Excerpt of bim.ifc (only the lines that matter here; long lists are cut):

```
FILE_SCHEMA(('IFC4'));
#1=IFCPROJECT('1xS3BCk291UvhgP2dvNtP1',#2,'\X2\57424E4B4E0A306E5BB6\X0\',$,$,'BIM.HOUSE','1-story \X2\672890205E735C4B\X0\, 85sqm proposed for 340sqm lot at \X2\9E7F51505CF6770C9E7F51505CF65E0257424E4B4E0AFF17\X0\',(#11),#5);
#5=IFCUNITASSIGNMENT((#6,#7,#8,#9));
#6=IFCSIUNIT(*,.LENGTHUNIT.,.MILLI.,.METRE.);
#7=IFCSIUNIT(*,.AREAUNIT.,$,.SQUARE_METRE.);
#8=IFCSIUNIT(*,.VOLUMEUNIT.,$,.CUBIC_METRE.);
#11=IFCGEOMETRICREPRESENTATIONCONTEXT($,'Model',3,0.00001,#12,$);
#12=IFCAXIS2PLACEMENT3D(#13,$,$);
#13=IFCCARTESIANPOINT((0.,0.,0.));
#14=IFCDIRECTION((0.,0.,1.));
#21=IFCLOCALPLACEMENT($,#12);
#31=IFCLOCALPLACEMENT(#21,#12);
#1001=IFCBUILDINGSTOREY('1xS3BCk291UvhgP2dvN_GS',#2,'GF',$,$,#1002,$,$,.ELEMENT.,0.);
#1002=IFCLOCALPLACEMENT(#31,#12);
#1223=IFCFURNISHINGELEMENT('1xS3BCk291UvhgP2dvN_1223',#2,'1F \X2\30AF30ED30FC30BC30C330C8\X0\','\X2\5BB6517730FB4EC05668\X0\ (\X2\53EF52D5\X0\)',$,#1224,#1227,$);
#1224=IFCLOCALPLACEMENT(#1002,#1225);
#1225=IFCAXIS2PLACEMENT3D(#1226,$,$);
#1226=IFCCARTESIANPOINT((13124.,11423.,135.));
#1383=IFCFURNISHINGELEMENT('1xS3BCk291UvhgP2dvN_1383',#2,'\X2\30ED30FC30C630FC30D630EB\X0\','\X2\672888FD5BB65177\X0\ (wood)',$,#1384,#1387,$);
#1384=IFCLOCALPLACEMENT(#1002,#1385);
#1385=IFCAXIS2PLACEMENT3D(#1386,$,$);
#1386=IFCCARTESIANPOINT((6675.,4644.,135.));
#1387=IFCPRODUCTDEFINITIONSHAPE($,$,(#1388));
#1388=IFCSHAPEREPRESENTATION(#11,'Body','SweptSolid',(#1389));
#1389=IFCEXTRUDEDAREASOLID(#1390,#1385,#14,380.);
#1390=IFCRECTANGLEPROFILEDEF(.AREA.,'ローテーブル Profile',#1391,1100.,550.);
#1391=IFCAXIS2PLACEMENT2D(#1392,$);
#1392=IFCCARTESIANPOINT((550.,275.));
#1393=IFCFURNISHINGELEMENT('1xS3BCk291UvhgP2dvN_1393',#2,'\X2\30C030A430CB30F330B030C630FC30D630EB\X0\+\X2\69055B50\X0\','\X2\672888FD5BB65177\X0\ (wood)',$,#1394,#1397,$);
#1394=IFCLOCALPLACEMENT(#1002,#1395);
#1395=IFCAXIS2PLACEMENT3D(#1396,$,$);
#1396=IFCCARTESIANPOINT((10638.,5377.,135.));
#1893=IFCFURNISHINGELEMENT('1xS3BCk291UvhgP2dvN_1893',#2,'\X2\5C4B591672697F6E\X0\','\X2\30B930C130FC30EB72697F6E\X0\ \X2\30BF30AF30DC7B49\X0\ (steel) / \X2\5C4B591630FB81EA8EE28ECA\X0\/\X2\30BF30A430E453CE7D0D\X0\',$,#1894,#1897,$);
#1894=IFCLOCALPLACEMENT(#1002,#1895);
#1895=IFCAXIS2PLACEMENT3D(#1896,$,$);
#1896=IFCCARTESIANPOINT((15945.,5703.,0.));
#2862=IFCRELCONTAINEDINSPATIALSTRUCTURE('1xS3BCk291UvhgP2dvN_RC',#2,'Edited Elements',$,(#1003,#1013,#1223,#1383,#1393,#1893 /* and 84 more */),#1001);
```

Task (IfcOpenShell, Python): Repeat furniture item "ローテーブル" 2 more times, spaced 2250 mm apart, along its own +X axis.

```python
import ifcopenshell
import ifcopenshell.api.geometry
import ifcopenshell.api.root
import ifcopenshell.util.element
import ifcopenshell.util.placement

model = ifcopenshell.open("bim.ifc")


def reuse_history(source, copy):
    """copy_class also copies each property set's owner history, people and application; keep the originals."""
    for rel in copy.IsDefinedBy:
        if rel.is_a("IfcRelDefinesByProperties") and (history := rel.RelatingPropertyDefinition.OwnerHistory):
            rel.RelatingPropertyDefinition.OwnerHistory = source.OwnerHistory
            ifcopenshell.util.element.remove_deep2(model, history)


source = model.by_guid("1xS3BCk291UvhgP2dvN_1383")
base = ifcopenshell.util.placement.get_local_placement(source.ObjectPlacement)
step = base[:3, 0] * 2250.0

for i in range(1, 3):
    copy = ifcopenshell.api.root.copy_class(model, product=source)
    copy.Representation = ifcopenshell.util.element.copy_deep(
        model, source.Representation, exclude=["IfcGeometricRepresentationContext", "IfcRepresentationMap"]
    )
    reuse_history(source, copy)
    matrix = base.copy()
    matrix[:3, 3] += i * step
    print("added at", matrix[:3, 3].round(3) + 0.0)
    ifcopenshell.api.geometry.edit_object_placement(model, product=copy, matrix=matrix, is_si=False)

model.write("bim_v2.ifc")
```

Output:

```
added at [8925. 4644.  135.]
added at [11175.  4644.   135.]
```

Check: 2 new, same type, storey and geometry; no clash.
